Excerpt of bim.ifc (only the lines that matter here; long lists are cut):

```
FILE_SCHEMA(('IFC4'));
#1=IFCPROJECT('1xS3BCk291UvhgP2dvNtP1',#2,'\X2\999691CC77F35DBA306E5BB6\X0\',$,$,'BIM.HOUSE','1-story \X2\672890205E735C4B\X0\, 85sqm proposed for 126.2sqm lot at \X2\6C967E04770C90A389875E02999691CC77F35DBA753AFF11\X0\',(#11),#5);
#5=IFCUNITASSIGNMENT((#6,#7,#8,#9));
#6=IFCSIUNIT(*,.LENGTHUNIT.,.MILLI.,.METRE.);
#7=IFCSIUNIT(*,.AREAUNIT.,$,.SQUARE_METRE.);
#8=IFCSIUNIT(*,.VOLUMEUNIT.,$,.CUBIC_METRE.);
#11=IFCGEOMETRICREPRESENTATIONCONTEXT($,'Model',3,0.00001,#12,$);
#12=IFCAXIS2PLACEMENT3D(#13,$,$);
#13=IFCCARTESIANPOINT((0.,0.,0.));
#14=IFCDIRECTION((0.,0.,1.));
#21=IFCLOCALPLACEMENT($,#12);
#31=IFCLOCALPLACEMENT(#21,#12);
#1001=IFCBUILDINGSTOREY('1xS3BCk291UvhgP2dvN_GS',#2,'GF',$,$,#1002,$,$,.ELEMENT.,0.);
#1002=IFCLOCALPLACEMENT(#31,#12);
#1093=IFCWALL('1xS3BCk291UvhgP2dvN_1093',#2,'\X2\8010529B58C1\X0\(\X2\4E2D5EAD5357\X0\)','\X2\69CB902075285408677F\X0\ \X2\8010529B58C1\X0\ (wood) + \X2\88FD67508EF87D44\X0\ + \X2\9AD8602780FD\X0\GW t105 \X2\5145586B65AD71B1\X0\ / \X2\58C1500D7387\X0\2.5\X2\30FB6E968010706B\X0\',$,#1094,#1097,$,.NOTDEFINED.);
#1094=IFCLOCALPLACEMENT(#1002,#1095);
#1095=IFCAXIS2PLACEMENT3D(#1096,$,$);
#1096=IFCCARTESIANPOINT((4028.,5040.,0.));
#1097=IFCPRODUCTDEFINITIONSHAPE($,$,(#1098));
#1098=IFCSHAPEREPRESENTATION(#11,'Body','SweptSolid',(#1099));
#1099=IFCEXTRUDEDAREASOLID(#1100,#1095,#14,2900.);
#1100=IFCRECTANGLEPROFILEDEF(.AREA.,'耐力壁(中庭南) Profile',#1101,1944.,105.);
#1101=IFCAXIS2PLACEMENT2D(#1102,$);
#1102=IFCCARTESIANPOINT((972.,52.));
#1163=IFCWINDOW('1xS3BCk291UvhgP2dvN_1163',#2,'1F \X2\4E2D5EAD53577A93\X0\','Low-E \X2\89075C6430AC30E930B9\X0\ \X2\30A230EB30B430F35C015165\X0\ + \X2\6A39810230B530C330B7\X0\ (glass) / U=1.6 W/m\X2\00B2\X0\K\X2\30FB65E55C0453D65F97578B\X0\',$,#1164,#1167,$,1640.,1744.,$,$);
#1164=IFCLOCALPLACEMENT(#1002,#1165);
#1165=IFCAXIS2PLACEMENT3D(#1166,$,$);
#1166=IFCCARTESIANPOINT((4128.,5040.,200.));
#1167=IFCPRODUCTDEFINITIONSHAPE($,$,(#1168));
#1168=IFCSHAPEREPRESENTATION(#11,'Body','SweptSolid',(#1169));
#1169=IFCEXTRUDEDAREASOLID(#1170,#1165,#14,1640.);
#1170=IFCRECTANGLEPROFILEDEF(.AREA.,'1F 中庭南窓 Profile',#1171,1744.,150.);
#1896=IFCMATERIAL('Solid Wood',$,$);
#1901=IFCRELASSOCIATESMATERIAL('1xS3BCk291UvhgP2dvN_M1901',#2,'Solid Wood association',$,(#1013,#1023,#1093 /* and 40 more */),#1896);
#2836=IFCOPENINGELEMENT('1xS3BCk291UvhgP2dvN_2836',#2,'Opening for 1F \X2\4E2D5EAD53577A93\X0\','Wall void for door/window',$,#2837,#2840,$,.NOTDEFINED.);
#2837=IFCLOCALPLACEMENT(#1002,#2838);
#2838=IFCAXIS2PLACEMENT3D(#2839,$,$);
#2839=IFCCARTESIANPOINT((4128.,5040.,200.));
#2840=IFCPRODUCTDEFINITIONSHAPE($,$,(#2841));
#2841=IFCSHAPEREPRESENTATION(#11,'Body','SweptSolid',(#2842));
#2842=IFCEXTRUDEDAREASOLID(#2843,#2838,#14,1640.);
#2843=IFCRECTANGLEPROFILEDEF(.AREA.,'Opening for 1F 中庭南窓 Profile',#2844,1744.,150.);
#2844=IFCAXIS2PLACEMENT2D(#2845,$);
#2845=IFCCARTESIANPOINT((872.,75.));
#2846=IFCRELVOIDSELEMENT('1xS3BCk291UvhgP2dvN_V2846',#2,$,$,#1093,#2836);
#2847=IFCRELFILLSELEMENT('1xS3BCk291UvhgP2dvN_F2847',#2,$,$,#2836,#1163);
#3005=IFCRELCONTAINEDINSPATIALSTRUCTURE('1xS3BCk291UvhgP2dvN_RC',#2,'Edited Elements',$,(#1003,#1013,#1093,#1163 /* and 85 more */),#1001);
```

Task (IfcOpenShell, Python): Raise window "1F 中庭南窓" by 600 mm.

```python
import numpy as np
import ifcopenshell
import ifcopenshell.api.geometry
import ifcopenshell.util.placement
import ifcopenshell.util.unit

model = ifcopenshell.open("bim.ifc")
unit_scale = ifcopenshell.util.unit.calculate_unit_scale(model)

window = model.by_guid("1xS3BCk291UvhgP2dvN_1163")
opening = window.FillsVoids[0].RelatingOpeningElement
dz = 600.0

shift = np.array([0.0, 0.0, dz])
# The window is not placed relative to its opening, so move both.
for product in (opening, window):
    matrix = ifcopenshell.util.placement.get_local_placement(product.ObjectPlacement)
    matrix[:3, 3] += shift
    ifcopenshell.api.geometry.edit_object_placement(model, product=product, matrix=matrix, is_si=False)

print(f"moved by {dz * unit_scale:+.3f} m")

model.write("bim_edited.ifc")
```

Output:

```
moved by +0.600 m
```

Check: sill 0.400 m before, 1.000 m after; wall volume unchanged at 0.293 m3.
